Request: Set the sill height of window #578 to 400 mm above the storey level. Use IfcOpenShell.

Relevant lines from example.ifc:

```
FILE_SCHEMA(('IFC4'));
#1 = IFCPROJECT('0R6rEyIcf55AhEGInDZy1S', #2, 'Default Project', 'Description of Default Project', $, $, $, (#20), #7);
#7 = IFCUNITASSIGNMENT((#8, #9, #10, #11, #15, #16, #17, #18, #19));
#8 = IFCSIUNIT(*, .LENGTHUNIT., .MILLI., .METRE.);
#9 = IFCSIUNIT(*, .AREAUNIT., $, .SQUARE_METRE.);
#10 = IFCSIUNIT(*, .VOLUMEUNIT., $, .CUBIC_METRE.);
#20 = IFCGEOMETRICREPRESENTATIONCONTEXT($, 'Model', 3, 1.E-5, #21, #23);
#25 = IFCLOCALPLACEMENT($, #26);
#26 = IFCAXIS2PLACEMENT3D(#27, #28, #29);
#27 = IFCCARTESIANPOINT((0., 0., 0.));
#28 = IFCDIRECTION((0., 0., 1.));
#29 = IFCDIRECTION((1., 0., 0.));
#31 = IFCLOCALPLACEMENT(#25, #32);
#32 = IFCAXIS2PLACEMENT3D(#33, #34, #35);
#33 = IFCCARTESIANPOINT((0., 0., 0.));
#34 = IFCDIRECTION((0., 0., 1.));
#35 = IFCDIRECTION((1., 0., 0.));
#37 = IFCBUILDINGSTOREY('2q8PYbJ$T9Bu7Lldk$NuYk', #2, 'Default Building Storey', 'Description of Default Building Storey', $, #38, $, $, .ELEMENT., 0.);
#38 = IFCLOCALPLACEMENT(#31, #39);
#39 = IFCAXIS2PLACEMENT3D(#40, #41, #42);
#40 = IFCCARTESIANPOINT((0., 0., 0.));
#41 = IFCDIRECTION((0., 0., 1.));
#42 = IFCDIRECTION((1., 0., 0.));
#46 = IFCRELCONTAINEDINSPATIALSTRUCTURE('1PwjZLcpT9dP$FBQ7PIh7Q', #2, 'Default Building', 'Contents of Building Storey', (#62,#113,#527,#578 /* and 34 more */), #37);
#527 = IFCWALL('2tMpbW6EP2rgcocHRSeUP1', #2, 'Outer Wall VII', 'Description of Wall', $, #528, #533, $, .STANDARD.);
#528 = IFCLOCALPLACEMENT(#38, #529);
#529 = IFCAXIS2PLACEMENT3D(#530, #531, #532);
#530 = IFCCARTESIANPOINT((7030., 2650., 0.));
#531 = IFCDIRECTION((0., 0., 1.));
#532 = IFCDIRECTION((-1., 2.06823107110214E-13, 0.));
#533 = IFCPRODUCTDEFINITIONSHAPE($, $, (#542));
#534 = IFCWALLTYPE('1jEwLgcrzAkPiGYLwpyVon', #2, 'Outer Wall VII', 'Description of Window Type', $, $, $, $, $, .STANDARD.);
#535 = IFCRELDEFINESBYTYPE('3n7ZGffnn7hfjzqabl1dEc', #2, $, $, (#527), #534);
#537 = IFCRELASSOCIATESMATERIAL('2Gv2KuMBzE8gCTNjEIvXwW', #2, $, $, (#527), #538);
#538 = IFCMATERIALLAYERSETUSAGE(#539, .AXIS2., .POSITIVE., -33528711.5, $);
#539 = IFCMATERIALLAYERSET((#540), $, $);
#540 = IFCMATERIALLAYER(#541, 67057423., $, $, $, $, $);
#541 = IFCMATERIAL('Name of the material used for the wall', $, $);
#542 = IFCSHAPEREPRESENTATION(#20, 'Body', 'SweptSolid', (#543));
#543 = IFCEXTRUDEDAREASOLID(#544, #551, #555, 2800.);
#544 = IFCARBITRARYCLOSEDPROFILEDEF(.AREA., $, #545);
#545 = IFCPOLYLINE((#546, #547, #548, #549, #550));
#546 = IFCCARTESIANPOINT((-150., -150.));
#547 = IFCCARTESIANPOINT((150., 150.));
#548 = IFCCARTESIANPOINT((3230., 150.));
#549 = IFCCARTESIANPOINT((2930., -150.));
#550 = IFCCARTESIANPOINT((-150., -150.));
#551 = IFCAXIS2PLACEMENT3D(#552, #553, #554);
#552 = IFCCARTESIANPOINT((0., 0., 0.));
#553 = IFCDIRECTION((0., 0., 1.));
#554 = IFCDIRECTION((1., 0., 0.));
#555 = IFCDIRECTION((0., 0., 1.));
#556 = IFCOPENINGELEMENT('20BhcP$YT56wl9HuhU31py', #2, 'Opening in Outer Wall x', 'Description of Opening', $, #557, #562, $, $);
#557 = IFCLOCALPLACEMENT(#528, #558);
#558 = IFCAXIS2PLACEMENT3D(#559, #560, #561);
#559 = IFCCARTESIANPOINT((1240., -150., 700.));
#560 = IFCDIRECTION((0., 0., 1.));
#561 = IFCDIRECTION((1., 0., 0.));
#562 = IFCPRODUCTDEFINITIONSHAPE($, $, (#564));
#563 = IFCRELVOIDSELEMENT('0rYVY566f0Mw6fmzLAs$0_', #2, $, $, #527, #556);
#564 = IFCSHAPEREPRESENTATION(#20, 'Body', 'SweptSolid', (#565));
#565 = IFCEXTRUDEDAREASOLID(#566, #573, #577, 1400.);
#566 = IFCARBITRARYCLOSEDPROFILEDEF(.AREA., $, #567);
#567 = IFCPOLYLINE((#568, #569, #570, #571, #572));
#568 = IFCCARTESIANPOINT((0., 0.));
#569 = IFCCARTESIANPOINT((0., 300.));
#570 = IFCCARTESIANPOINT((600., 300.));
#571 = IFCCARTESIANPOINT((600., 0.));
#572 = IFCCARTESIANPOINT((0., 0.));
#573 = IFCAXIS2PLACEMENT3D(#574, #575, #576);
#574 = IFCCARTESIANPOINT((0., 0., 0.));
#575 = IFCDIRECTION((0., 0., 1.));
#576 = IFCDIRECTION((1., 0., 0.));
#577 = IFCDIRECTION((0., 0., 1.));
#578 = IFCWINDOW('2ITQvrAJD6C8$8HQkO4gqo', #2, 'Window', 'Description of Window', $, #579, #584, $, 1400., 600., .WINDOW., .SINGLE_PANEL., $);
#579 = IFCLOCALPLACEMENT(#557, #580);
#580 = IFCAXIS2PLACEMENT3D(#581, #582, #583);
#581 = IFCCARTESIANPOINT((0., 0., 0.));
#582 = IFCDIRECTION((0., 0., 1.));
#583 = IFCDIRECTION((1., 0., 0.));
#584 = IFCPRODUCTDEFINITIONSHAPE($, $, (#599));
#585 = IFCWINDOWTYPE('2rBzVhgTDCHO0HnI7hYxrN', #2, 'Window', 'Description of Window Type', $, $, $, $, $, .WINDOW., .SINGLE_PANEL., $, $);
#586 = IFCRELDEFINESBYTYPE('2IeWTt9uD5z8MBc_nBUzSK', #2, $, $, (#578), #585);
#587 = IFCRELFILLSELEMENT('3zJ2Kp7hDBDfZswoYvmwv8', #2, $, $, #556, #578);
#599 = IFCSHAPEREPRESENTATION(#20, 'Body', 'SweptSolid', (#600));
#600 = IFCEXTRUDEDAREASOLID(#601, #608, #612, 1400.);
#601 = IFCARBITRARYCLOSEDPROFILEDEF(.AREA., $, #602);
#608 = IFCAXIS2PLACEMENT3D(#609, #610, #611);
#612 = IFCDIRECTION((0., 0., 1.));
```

```python
import numpy as np
import ifcopenshell
import ifcopenshell.api.geometry
import ifcopenshell.geom
import ifcopenshell.util.element
import ifcopenshell.util.placement
import ifcopenshell.util.shape
import ifcopenshell.util.unit

model = ifcopenshell.open("example.ifc")
unit_scale = ifcopenshell.util.unit.calculate_unit_scale(model)

window = model.by_guid("2ITQvrAJD6C8$8HQkO4gqo")
opening = window.FillsVoids[0].RelatingOpeningElement
storey = ifcopenshell.util.element.get_container(window, ifc_class="IfcBuildingStorey")
level = ifcopenshell.util.placement.get_local_placement(storey.ObjectPlacement)[2, 3]

# The opening's origin need not be at the sill, so measure its lowest point.
shape = ifcopenshell.geom.create_shape(ifcopenshell.geom.settings(), opening)
bottom = ifcopenshell.util.shape.get_shape_bottom_elevation(shape, shape.geometry) / unit_scale
dz = level + 0.4 / unit_scale - bottom

shift = np.array([0.0, 0.0, dz])
# The window is placed relative to its opening, so it follows when the opening moves.
matrix = ifcopenshell.util.placement.get_local_placement(opening.ObjectPlacement)
matrix[:3, 3] += shift
ifcopenshell.api.geometry.edit_object_placement(
    model, product=opening, matrix=matrix, is_si=False, should_transform_children=True
)

print(f"moved by {dz * unit_scale:+.3f} m")

model.write("example_rev.ifc")
```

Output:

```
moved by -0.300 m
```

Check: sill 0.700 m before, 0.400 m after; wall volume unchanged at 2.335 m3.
